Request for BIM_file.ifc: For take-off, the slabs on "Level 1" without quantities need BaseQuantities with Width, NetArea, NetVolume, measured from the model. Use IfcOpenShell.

First a look at what the model holds.

```python
import ifcopenshell
import ifcopenshell.util.element
import ifcopenshell.util.unit

model = ifcopenshell.open("BIM_file.ifc")
print(model.schema)
for unit_type in ("LENGTHUNIT", "AREAUNIT", "VOLUMEUNIT"):
    print(unit_type, ifcopenshell.util.unit.calculate_unit_scale(model, unit_type))
storey = next(s for s in model.by_type("IfcBuildingStorey") if s.Name == "Level 1")
slabs = [e for e in ifcopenshell.util.element.get_decomposition(storey) if e.is_a("IfcSlab")]
for e in sorted(slabs, key=lambda e: e.id()):
    print(e.id(), e.is_a(), e.Name, list(ifcopenshell.util.element.get_psets(e, qtos_only=True)), sep=" | ")
```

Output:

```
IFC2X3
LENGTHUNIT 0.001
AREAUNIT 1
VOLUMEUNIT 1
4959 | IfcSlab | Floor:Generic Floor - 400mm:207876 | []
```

```python
import ifcopenshell
import ifcopenshell.api.pset
import ifcopenshell.geom
import ifcopenshell.util.element
import ifcopenshell.util.shape
import ifcopenshell.util.unit

model = ifcopenshell.open("BIM_file.ifc")
unit_scale = ifcopenshell.util.unit.calculate_unit_scale(model)
area_scale = ifcopenshell.util.unit.calculate_unit_scale(model, "AREAUNIT")
volume_scale = ifcopenshell.util.unit.calculate_unit_scale(model, "VOLUMEUNIT")
settings = ifcopenshell.geom.settings()

storey = next(s for s in model.by_type("IfcBuildingStorey") if s.Name == "Level 1")
slabs = [e for e in ifcopenshell.util.element.get_decomposition(storey) if e.is_a("IfcSlab")]

for e in sorted(slabs, key=lambda e: e.id()):
    if ifcopenshell.util.element.get_psets(e, qtos_only=True, should_inherit=False):
        continue
    # Geometry comes back in metres, in the element's own axes.
    shape = ifcopenshell.geom.create_shape(settings, e)
    values = {
        "Width": ifcopenshell.util.shape.get_z(shape.geometry) / unit_scale,
        "NetArea": ifcopenshell.util.shape.get_footprint_area(shape.geometry) / area_scale,
        "NetVolume": ifcopenshell.util.shape.get_volume(shape.geometry) / volume_scale,
    }
    qto = ifcopenshell.api.pset.add_qto(model, product=e, name="BaseQuantities")
    ifcopenshell.api.pset.edit_qto(model, qto=qto, properties=values)
    print(e.id(), {k: round(v, 3) for k, v in values.items()})

model.write("BIM_file_edited.ifc")
```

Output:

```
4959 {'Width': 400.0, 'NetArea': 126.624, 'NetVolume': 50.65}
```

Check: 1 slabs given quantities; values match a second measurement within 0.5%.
